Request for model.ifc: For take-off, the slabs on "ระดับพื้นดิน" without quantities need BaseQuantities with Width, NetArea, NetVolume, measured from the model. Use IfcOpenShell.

First a look at what the model holds.

```python
import ifcopenshell
import ifcopenshell.util.element
import ifcopenshell.util.unit

model = ifcopenshell.open("model.ifc")
print(model.schema)
for unit_type in ("LENGTHUNIT", "AREAUNIT", "VOLUMEUNIT"):
    print(unit_type, ifcopenshell.util.unit.calculate_unit_scale(model, unit_type))
storey = next(s for s in model.by_type("IfcBuildingStorey") if s.Name == "ระดับพื้นดิน")
slabs = [e for e in ifcopenshell.util.element.get_decomposition(storey) if e.is_a("IfcSlab")]
for e in sorted(slabs, key=lambda e: e.id()):
    print(e.id(), e.is_a(), e.Name, list(ifcopenshell.util.element.get_psets(e, qtos_only=True)), sep=" | ")
```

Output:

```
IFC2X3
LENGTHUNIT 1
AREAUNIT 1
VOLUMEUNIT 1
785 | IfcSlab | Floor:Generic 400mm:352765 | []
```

```python
import ifcopenshell
import ifcopenshell.api.pset
import ifcopenshell.geom
import ifcopenshell.util.element
import ifcopenshell.util.shape
import ifcopenshell.util.unit

model = ifcopenshell.open("model.ifc")
unit_scale = ifcopenshell.util.unit.calculate_unit_scale(model)
area_scale = ifcopenshell.util.unit.calculate_unit_scale(model, "AREAUNIT")
volume_scale = ifcopenshell.util.unit.calculate_unit_scale(model, "VOLUMEUNIT")
settings = ifcopenshell.geom.settings()

storey = next(s for s in model.by_type("IfcBuildingStorey") if s.Name == "ระดับพื้นดิน")
slabs = [e for e in ifcopenshell.util.element.get_decomposition(storey) if e.is_a("IfcSlab")]

for e in sorted(slabs, key=lambda e: e.id()):
    if ifcopenshell.util.element.get_psets(e, qtos_only=True, should_inherit=False):
        continue
    # Geometry comes back in metres, in the element's own axes.
    shape = ifcopenshell.geom.create_shape(settings, e)
    values = {
        "Width": ifcopenshell.util.shape.get_z(shape.geometry) / unit_scale,
        "NetArea": ifcopenshell.util.shape.get_footprint_area(shape.geometry) / area_scale,
        "NetVolume": ifcopenshell.util.shape.get_volume(shape.geometry) / volume_scale,
    }
    qto = ifcopenshell.api.pset.add_qto(model, product=e, name="BaseQuantities")
    ifcopenshell.api.pset.edit_qto(model, qto=qto, properties=values)
    print(e.id(), {k: round(v, 3) for k, v in values.items()})

model.write("model_rev.ifc")
```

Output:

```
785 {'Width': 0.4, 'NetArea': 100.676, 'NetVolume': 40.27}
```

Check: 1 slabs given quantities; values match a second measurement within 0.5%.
